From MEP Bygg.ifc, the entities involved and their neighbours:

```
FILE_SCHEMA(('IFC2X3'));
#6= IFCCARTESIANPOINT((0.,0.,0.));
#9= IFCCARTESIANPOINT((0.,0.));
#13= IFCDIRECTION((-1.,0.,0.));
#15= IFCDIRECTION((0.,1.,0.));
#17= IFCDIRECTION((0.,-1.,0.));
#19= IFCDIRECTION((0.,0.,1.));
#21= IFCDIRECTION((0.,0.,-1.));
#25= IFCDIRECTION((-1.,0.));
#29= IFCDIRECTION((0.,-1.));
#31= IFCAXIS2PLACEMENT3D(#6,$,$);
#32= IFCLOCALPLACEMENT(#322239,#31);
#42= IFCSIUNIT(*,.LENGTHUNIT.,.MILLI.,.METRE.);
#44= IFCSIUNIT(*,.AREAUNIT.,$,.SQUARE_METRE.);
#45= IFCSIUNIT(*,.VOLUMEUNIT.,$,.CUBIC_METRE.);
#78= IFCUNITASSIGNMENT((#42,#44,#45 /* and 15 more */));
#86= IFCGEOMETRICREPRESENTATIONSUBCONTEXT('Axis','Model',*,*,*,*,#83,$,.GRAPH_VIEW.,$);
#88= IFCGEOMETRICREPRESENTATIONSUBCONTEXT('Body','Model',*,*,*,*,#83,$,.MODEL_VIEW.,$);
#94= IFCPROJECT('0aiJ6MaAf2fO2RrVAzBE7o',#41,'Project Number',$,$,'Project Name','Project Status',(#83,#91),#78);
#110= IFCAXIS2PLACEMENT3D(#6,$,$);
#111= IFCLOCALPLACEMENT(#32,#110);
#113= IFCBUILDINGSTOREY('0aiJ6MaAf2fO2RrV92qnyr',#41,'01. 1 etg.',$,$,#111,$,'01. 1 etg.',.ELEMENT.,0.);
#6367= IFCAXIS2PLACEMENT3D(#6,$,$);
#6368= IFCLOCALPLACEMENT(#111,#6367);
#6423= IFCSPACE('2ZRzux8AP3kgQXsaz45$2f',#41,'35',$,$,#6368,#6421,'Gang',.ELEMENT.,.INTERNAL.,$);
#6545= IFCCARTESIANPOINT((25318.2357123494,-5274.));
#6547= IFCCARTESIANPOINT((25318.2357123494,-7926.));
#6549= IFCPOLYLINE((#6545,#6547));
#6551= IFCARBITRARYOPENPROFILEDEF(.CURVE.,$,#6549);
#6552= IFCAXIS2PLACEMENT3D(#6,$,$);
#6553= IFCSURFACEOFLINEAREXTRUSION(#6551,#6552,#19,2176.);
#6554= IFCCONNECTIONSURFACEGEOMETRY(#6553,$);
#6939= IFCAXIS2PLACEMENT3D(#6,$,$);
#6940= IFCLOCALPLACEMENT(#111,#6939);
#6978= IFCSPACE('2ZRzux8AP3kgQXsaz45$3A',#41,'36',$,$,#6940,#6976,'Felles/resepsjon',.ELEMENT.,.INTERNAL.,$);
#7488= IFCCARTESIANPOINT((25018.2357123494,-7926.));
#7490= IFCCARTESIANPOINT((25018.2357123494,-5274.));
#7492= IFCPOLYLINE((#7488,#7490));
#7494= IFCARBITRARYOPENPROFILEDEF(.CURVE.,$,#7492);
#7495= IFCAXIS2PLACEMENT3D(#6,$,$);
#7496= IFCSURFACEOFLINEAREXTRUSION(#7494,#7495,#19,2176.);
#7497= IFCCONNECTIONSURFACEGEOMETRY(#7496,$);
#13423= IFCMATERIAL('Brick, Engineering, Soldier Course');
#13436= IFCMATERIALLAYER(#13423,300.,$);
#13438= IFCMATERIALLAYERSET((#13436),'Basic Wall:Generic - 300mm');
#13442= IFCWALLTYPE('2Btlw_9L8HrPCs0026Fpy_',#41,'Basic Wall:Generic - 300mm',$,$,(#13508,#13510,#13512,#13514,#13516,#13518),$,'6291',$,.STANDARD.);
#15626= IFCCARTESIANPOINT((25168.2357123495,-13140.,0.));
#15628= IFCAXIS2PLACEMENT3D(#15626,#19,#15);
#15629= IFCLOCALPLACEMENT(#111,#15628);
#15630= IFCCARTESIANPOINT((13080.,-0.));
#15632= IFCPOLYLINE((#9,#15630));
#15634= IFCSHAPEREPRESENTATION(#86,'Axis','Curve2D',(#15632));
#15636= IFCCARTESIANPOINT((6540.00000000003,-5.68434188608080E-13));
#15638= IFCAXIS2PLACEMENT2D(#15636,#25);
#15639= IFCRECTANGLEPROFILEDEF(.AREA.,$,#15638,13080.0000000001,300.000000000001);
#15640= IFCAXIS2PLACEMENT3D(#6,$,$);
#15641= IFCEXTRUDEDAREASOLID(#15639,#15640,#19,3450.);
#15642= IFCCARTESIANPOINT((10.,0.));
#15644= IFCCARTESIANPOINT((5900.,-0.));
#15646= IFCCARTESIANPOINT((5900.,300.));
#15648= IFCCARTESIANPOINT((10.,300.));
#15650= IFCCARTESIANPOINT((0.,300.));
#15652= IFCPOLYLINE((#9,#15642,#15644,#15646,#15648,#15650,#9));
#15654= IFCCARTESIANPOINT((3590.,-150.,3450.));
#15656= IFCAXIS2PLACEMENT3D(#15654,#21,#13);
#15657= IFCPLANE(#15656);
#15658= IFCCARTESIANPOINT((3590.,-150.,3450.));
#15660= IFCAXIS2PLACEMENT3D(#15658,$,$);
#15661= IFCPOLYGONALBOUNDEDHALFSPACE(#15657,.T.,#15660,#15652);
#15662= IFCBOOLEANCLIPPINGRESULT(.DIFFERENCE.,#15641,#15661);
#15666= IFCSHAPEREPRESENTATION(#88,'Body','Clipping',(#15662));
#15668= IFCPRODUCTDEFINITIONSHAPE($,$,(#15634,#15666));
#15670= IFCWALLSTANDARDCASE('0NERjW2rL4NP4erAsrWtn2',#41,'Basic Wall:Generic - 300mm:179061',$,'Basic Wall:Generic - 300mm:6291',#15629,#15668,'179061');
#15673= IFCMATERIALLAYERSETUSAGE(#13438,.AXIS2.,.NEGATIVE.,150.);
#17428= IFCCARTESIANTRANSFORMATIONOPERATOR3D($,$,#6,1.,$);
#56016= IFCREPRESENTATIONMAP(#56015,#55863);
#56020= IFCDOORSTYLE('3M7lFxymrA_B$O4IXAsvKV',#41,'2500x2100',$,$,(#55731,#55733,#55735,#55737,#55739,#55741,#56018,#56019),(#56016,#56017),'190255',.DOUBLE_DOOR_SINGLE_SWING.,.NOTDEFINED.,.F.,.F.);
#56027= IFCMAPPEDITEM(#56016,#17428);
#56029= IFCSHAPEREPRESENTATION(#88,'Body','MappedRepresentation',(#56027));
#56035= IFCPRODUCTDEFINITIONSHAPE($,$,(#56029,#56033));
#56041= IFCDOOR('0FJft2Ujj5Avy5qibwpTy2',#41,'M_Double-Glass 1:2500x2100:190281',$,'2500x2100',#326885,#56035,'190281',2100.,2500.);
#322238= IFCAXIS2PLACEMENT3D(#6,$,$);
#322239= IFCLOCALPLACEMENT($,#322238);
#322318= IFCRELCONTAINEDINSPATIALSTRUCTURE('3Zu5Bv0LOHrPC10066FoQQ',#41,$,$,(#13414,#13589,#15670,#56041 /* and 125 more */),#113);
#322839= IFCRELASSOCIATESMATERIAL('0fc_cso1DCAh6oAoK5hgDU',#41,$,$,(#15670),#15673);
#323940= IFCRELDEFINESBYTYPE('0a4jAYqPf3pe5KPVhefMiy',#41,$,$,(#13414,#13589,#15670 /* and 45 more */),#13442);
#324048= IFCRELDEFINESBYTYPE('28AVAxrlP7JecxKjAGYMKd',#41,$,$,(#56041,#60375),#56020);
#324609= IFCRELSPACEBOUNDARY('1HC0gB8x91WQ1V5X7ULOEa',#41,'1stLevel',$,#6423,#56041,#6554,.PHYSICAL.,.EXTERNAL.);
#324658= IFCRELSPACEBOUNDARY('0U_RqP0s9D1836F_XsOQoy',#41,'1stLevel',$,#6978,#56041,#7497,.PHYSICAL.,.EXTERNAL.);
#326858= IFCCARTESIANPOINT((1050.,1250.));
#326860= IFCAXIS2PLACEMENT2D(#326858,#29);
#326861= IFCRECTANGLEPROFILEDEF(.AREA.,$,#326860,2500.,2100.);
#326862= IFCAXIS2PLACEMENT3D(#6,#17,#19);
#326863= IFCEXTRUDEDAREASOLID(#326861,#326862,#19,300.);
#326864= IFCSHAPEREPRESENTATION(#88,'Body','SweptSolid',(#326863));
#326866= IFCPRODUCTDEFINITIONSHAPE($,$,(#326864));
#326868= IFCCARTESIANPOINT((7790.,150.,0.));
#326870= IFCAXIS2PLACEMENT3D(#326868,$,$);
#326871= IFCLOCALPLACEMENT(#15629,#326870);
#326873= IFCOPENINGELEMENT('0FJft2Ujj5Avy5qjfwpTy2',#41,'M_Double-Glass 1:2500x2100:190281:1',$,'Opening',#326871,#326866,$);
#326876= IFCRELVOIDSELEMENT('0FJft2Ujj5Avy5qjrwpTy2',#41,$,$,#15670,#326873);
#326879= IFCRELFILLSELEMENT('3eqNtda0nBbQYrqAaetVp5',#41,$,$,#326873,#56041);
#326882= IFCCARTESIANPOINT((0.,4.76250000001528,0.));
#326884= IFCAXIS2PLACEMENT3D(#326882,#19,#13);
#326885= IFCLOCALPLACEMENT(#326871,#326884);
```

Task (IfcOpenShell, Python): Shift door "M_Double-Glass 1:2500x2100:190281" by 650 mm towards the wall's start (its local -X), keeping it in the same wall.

```python
import numpy as np
import ifcopenshell
import ifcopenshell.api.geometry
import ifcopenshell.util.placement

model = ifcopenshell.open("MEP Bygg.ifc")

door = model.by_guid("0FJft2Ujj5Avy5qibwpTy2")
opening = door.FillsVoids[0].RelatingOpeningElement
wall = opening.VoidsElements[0].RelatingBuildingElement

wall_matrix = ifcopenshell.util.placement.get_local_placement(wall.ObjectPlacement)
shift = wall_matrix[:3, 0] * -650.0
before = ifcopenshell.util.placement.get_local_placement(door.ObjectPlacement)[:3, 3].copy()

# The door is placed relative to its opening, so it follows when the opening moves.
matrix = ifcopenshell.util.placement.get_local_placement(opening.ObjectPlacement)
matrix[:3, 3] += shift
ifcopenshell.api.geometry.edit_object_placement(
    model, product=opening, matrix=matrix, is_si=False, should_transform_children=True
)

# Space boundary surfaces are stored in each space's coordinates; move them too.
for rel in door.ProvidesBoundaries:
    if not rel.ConnectionGeometry:
        continue
    surface = rel.ConnectionGeometry.SurfaceOnRelatingElement
    space_matrix = ifcopenshell.util.placement.get_local_placement(rel.RelatingSpace.ObjectPlacement)
    point = np.array(surface.Position.Location.Coordinates) + space_matrix[:3, :3].T @ shift
    surface.Position = model.createIfcAxis2Placement3D(
        model.createIfcCartesianPoint(point.tolist()), surface.Position.Axis, surface.Position.RefDirection
    )

after = ifcopenshell.util.placement.get_local_placement(door.ObjectPlacement)[:3, 3]
print("door moved by", (after - before).round(3) + 0.0)

model.write("MEP Bygg_updated.ifc")
```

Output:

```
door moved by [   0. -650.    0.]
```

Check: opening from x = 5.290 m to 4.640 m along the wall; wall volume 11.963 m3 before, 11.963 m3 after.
